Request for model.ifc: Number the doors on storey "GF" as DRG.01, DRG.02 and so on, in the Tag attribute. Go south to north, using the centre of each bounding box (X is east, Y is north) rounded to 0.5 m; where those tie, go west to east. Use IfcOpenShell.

First a look at what the model holds.

```python
import ifcopenshell
import ifcopenshell.util.element
import ifcopenshell.util.placement

model = ifcopenshell.open("model.ifc")
print(model.schema)
storey = next(s for s in model.by_type("IfcBuildingStorey") if s.Name == "GF")
doors = [e for e in ifcopenshell.util.element.get_decomposition(storey) if e.is_a("IfcDoor")]
for e in sorted(doors, key=lambda e: e.id()):
    origin = ifcopenshell.util.placement.get_local_placement(e.ObjectPlacement)[:3, 3]
    print(e.id(), e.Tag, e.Name, origin.round(2) + 0.0, sep=" | ")
```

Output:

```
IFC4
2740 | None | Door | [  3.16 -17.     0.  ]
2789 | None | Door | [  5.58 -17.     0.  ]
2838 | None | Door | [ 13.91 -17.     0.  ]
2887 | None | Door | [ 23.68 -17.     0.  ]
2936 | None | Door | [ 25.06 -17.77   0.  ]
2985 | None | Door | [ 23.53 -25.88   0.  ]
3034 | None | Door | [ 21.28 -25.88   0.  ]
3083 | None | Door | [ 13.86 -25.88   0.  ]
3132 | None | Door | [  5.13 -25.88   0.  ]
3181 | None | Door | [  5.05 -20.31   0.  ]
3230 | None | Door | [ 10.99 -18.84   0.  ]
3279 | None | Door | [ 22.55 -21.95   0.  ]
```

```python
import ifcopenshell
import ifcopenshell.geom
import ifcopenshell.util.element
import ifcopenshell.util.shape

model = ifcopenshell.open("model.ifc")
settings = ifcopenshell.geom.settings()
settings.set("use-world-coords", True)


def centre(element):
    shape = ifcopenshell.geom.create_shape(settings, element)
    return ifcopenshell.util.shape.get_bbox_centroid(shape.geometry)


storey = next(s for s in model.by_type("IfcBuildingStorey") if s.Name == "GF")
doors = [e for e in ifcopenshell.util.element.get_decomposition(storey) if e.is_a("IfcDoor")]

# Insertion points can sit at a corner or the storey origin, so sort by the geometry (in metres).
centres = {e: centre(e) for e in doors}
doors.sort(key=lambda e: (round(centres[e][1] / 0.5), centres[e][0]))

for i, e in enumerate(doors, start=1):
    number = f"DRG.{i:02d}"
    e.Tag = number
    print(e.id(), number)

model.write("model-out.ifc")
```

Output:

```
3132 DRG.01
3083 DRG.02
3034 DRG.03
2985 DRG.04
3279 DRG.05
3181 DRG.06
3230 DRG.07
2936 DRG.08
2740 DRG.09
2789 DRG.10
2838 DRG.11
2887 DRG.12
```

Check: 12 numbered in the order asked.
